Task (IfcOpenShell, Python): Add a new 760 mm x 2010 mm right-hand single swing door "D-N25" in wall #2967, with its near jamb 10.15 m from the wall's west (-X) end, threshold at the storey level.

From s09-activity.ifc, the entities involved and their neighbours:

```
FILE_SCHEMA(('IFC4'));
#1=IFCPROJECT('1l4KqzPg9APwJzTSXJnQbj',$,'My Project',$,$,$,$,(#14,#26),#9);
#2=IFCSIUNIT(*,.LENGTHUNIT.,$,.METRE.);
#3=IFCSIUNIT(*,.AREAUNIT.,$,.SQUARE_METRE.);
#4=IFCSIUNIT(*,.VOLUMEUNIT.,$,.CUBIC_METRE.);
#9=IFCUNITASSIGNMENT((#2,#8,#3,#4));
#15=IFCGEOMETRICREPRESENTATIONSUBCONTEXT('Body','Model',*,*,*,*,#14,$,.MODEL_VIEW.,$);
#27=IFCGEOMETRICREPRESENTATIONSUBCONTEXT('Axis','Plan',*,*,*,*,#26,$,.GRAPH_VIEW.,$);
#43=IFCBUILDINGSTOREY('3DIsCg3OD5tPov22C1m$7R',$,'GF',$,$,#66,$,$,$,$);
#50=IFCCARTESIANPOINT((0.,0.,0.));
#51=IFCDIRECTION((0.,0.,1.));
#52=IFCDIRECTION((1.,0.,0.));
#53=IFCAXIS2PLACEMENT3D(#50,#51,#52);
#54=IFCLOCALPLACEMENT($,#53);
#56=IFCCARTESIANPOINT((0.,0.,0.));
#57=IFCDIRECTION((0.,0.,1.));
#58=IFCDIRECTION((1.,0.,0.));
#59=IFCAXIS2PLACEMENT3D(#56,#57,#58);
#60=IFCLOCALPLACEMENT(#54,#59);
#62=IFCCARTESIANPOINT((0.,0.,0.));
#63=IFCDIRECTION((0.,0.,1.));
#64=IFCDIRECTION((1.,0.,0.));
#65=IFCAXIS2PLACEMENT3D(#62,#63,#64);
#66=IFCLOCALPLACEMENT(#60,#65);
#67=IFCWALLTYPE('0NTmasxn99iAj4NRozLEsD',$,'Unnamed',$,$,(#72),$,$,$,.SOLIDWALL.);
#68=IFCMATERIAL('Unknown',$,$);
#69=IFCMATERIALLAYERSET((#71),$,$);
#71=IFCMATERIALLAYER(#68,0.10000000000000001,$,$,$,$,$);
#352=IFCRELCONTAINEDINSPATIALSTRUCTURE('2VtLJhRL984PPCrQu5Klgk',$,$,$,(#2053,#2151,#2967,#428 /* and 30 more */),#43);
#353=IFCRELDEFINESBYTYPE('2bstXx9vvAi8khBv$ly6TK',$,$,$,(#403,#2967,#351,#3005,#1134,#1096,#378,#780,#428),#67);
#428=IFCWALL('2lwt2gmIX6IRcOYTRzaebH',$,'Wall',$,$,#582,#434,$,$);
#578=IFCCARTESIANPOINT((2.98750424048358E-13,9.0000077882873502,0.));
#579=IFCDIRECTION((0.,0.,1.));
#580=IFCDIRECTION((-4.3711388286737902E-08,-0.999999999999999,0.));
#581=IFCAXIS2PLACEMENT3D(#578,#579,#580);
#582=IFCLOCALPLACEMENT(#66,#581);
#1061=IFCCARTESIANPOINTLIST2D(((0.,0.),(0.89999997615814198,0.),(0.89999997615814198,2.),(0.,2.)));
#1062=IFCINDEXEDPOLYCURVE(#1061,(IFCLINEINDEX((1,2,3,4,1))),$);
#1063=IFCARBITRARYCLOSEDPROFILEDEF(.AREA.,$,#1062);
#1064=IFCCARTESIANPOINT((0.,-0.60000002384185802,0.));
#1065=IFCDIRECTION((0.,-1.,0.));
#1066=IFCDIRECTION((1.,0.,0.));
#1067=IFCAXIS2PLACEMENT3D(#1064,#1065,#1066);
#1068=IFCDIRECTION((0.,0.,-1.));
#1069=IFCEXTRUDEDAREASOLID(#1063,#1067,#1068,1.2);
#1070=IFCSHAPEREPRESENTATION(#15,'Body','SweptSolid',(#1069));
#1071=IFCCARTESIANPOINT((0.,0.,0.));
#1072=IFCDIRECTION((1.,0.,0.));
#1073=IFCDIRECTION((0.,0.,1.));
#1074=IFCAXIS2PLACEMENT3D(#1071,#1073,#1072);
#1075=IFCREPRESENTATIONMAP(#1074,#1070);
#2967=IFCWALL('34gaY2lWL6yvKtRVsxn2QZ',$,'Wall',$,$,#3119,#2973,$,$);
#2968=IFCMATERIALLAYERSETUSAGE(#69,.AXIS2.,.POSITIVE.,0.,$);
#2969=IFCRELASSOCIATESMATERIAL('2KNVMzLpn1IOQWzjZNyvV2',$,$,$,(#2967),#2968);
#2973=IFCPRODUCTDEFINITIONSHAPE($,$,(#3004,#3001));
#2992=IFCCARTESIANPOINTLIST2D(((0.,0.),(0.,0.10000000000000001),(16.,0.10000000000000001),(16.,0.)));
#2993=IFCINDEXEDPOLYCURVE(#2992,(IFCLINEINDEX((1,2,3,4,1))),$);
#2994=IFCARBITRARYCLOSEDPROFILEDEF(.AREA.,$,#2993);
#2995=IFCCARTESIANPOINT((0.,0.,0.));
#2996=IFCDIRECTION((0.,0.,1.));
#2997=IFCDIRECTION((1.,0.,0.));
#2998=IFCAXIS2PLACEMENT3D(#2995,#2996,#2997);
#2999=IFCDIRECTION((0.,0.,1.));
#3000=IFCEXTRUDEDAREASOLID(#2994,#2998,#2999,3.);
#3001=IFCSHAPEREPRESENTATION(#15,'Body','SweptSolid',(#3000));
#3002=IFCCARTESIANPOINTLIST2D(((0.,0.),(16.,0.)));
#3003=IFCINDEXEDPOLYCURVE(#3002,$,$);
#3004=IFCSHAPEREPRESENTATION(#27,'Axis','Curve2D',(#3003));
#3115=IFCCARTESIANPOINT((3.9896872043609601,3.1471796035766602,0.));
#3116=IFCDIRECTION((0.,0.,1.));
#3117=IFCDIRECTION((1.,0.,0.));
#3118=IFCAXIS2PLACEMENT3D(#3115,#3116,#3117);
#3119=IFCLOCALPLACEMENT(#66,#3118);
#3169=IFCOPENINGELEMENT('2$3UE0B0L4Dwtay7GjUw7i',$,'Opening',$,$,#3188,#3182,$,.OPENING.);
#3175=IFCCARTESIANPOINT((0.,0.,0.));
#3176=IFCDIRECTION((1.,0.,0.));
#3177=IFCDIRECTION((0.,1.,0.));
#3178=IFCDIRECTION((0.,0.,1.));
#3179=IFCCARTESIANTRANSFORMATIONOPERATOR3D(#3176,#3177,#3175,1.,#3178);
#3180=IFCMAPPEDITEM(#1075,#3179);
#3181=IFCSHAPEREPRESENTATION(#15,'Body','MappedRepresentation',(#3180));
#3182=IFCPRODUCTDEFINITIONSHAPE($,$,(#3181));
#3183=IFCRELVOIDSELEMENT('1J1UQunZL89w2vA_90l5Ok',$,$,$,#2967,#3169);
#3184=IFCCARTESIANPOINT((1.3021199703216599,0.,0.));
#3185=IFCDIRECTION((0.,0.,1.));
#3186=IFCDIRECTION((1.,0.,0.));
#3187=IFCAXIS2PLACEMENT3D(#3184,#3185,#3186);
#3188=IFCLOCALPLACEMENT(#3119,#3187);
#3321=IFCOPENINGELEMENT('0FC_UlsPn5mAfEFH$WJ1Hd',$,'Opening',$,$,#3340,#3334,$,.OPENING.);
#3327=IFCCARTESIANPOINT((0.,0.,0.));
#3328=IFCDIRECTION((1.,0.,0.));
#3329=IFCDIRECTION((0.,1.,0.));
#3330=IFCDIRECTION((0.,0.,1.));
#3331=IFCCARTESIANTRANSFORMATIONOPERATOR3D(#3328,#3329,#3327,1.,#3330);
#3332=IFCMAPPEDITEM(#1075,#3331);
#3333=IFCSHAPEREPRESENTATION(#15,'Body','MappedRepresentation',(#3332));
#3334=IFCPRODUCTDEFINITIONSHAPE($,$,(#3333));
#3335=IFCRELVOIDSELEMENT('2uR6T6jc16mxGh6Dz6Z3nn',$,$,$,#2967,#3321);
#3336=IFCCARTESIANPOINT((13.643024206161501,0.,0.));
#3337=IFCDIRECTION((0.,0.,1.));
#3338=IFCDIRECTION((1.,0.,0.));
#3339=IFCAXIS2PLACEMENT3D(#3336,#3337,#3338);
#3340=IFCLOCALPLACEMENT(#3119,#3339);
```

```python
import numpy as np
import ifcopenshell
import ifcopenshell.api.feature
import ifcopenshell.api.geometry
import ifcopenshell.api.root
import ifcopenshell.api.spatial
import ifcopenshell.geom
import ifcopenshell.util.element
import ifcopenshell.util.placement
import ifcopenshell.util.representation
import ifcopenshell.util.shape
import ifcopenshell.util.unit

model = ifcopenshell.open("s09-activity.ifc")
unit_scale = ifcopenshell.util.unit.calculate_unit_scale(model)
settings = ifcopenshell.geom.settings()


def volume(element):
    """Net volume in cubic metres, openings subtracted."""
    shape = ifcopenshell.geom.create_shape(settings, element)
    return ifcopenshell.util.shape.get_volume(shape.geometry)


wall = model.by_guid("34gaY2lWL6yvKtRVsxn2QZ")
storey = ifcopenshell.util.element.get_container(wall, ifc_class="IfcBuildingStorey")
context = ifcopenshell.util.representation.get_context(model, "Model", "Body", "MODEL_VIEW")
before = volume(wall)

width, height, from_end, sill = 0.76, 2.01, 10.15, 0.0  # metres

# The wall runs along its own X axis, and the end named is its -X end.
wall_shape = ifcopenshell.geom.create_shape(settings, wall)
x, y, z = ifcopenshell.util.shape.get_vertices(wall_shape.geometry).T
start = x.min() + from_end
face, thickness = float(y.min()), float(y.max() - y.min())
wall_matrix = ifcopenshell.util.placement.get_local_placement(wall.ObjectPlacement)
level = ifcopenshell.util.placement.get_local_placement(storey.ObjectPlacement)[2, 3]


def in_wall(x, y):
    """Placement at x, y metres in the wall's axes, at sill height."""
    matrix = wall_matrix.copy()
    matrix[:, 3] = wall_matrix @ np.array([x / unit_scale, y / unit_scale, 0.0, 1.0])
    matrix[2, 3] = level + sill / unit_scale
    return matrix


# Opening: a box that overshoots both wall faces by 50 mm.
opening = ifcopenshell.api.root.create_entity(model, ifc_class="IfcOpeningElement", predefined_type="OPENING")
box = ifcopenshell.api.geometry.add_wall_representation(
    model, context=context, length=width, height=height, thickness=thickness + 0.1
)
ifcopenshell.api.geometry.assign_representation(model, product=opening, representation=box)
ifcopenshell.api.geometry.edit_object_placement(model, product=opening, matrix=in_wall(start, face - 0.05), is_si=False)
ifcopenshell.api.feature.add_feature(model, feature=opening, element=wall)

door = ifcopenshell.api.root.create_entity(model, ifc_class="IfcDoor", name="D-N25", predefined_type="DOOR")
door.OverallWidth, door.OverallHeight = width / unit_scale, height / unit_scale
door.OperationType = "SINGLE_SWING_RIGHT"
body = ifcopenshell.api.geometry.add_door_representation(
    model,
    context=context,
    overall_width=door.OverallWidth,
    overall_height=door.OverallHeight,
    operation_type="SINGLE_SWING_RIGHT",
    lining_properties={"LiningDepth": thickness / unit_scale, "ThresholdDepth": thickness / unit_scale},
)
ifcopenshell.api.geometry.assign_representation(model, product=door, representation=body)
ifcopenshell.api.spatial.assign_container(model, products=[door], relating_structure=storey)
ifcopenshell.api.feature.add_filling(model, opening=opening, element=door)

# The lining spans the wall, so the door starts at the wall face.
ifcopenshell.api.geometry.edit_object_placement(model, product=door, matrix=in_wall(start, face), is_si=False)

after = volume(wall)

print(f"wall volume {before:.3f} -> {after:.3f} m3")

model.write("s09-activity_rev.ifc")
```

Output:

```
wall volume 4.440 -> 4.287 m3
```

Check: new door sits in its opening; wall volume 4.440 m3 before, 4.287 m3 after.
